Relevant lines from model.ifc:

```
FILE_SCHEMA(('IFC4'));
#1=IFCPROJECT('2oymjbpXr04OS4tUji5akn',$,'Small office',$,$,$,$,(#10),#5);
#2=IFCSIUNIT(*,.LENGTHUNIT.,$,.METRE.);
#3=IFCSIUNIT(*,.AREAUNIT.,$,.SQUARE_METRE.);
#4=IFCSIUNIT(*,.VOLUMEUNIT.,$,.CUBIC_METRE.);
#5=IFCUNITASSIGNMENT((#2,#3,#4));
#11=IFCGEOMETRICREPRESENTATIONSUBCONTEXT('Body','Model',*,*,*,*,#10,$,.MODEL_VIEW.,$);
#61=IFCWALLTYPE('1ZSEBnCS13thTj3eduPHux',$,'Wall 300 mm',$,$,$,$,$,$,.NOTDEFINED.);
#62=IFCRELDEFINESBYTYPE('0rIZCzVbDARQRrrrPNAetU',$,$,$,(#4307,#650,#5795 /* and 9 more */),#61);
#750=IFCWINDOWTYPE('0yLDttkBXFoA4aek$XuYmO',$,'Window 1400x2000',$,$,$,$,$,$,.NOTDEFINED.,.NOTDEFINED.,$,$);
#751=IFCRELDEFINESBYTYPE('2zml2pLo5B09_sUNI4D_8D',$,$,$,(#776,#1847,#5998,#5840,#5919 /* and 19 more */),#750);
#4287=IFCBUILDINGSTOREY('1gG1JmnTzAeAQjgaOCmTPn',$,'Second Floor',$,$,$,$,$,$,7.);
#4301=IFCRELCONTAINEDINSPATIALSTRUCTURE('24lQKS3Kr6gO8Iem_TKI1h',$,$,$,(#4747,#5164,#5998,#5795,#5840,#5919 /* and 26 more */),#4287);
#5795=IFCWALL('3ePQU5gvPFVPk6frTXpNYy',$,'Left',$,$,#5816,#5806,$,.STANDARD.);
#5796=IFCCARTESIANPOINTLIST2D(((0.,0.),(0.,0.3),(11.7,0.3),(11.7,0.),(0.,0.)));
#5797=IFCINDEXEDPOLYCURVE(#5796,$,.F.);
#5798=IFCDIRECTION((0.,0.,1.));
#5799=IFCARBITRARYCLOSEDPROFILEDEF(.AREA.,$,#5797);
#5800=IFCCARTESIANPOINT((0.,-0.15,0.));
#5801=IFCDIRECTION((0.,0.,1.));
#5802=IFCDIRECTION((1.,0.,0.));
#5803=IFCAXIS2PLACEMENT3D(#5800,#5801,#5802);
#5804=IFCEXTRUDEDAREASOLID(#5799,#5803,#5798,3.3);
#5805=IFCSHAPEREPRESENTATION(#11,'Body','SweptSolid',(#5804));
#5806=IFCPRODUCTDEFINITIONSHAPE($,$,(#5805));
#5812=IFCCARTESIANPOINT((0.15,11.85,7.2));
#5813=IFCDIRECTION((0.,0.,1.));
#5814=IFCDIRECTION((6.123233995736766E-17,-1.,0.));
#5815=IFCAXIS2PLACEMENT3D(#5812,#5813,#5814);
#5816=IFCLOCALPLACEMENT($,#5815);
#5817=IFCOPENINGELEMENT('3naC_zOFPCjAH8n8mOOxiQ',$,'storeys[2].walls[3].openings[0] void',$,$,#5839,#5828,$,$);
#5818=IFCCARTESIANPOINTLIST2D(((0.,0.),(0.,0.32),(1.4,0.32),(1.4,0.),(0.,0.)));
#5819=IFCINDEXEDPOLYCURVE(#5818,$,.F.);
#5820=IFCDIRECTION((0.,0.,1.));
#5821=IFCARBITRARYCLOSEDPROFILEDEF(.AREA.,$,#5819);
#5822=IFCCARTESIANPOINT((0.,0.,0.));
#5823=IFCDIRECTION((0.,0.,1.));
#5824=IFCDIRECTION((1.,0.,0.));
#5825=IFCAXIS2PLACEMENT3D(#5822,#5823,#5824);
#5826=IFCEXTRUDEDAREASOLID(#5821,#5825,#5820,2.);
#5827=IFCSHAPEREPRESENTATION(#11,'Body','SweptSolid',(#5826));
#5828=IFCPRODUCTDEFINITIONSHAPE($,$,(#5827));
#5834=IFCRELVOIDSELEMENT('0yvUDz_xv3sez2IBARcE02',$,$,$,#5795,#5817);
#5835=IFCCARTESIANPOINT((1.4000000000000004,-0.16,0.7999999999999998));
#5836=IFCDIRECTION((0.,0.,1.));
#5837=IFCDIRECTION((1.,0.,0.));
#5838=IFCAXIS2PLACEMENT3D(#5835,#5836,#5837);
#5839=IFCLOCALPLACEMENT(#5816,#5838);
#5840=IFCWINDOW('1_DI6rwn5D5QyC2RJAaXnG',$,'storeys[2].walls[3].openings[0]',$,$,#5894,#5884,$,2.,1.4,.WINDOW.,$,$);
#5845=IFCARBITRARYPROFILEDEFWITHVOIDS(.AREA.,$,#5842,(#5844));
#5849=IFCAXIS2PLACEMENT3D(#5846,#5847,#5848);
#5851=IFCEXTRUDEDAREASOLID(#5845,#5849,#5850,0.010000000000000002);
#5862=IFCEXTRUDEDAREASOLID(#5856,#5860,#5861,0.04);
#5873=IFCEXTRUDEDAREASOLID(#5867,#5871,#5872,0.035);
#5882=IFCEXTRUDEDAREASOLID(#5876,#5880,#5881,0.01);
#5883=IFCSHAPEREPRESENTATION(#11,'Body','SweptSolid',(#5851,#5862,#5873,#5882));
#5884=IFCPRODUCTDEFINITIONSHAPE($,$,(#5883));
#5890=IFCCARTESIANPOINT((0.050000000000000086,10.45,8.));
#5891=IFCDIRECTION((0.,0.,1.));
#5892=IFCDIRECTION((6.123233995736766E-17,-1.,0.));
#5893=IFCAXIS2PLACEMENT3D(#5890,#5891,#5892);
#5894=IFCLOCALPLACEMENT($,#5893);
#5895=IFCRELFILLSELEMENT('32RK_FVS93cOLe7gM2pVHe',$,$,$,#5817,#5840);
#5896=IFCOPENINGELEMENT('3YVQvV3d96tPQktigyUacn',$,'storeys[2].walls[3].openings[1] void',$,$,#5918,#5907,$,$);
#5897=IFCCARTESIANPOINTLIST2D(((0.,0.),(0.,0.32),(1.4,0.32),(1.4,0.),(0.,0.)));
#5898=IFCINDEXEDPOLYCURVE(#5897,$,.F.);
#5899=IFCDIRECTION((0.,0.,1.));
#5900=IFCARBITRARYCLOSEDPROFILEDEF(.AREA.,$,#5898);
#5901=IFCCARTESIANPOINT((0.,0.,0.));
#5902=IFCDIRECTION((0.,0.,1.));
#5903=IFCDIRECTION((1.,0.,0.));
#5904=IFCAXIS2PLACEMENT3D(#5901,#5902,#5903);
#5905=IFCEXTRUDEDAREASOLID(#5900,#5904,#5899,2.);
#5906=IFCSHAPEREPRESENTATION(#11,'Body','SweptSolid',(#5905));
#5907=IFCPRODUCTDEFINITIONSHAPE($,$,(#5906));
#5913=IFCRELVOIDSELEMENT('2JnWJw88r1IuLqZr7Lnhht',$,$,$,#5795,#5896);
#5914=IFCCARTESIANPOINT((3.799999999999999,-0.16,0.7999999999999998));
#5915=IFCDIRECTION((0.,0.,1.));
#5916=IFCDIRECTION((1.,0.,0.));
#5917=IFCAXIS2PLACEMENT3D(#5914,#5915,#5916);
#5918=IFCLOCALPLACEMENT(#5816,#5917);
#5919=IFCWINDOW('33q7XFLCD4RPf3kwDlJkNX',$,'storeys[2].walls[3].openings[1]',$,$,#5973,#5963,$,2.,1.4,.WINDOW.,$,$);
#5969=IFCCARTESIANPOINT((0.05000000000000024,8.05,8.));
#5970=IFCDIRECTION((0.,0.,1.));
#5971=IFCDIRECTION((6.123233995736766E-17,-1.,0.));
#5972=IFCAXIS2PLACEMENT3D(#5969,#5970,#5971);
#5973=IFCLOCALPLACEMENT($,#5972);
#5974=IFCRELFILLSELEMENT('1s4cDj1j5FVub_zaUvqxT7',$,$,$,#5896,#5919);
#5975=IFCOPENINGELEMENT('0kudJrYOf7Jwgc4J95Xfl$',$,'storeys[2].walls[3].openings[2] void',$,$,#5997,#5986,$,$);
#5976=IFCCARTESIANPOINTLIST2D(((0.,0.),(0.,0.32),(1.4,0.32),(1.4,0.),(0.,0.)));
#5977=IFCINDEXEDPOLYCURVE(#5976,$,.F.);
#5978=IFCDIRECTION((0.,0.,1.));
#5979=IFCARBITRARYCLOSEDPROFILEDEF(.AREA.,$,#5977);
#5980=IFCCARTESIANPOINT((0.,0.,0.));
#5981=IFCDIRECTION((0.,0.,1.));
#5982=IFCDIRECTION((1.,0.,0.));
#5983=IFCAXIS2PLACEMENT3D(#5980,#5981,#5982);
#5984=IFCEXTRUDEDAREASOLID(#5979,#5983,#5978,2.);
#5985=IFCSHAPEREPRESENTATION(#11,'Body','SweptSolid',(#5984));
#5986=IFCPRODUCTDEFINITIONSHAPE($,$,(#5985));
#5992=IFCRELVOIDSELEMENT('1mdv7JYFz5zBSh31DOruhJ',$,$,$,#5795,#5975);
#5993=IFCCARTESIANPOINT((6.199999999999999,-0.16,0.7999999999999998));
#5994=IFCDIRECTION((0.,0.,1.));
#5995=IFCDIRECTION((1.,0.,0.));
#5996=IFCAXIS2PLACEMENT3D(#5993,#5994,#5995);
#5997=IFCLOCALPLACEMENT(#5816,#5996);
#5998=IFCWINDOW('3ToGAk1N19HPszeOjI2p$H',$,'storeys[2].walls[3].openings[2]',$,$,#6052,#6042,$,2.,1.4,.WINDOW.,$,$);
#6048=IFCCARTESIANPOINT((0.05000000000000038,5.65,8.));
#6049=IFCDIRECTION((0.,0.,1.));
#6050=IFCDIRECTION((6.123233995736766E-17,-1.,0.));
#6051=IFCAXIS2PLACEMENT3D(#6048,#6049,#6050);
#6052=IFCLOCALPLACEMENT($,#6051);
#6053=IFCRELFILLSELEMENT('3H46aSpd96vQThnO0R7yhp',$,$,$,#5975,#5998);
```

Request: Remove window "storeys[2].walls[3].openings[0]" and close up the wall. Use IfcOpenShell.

```python
import ifcopenshell
import ifcopenshell.api.feature
import ifcopenshell.api.root
import ifcopenshell.geom
import ifcopenshell.util.shape

model = ifcopenshell.open("model.ifc")
settings = ifcopenshell.geom.settings()


def volume(element):
    """Net volume in cubic metres, openings subtracted."""
    shape = ifcopenshell.geom.create_shape(settings, element)
    return ifcopenshell.util.shape.get_volume(shape.geometry)


window = model.by_guid("1_DI6rwn5D5QyC2RJAaXnG")
opening = window.FillsVoids[0].RelatingOpeningElement
wall = opening.VoidsElements[0].RelatingBuildingElement
before = volume(wall)

ifcopenshell.api.root.remove_product(model, product=window)
ifcopenshell.api.feature.remove_feature(model, feature=opening)

after = volume(wall)

print(f"wall volume {before:.3f} -> {after:.3f} m3")

model.write("model_v2.ifc")
```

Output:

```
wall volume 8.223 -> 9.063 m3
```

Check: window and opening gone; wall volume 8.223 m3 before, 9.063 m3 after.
